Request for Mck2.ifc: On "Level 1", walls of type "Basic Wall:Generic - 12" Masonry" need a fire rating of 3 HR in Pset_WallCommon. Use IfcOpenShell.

First a look at what the model holds.

```python
import ifcopenshell
import ifcopenshell.util.element

model = ifcopenshell.open("Mck2.ifc")
print(model.schema)
storey = next(s for s in model.by_type("IfcBuildingStorey") if s.Name == "Level 1")
walls = [e for e in ifcopenshell.util.element.get_decomposition(storey) if e.is_a("IfcWall")]
seen = {}
for e in walls:
    element_type = ifcopenshell.util.element.get_type(e)
    key = (element_type.Name if element_type != e and element_type else None, ifcopenshell.util.element.get_pset(e, "Pset_WallCommon", "FireRating"))
    seen[key] = seen.get(key, 0) + 1
for (name, value), count in sorted(seen.items(), key=str):
    print(count, "x", name, "|", value)
```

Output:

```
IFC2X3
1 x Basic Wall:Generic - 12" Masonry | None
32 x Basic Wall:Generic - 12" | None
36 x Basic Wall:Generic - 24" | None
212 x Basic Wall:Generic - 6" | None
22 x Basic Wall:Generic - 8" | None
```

```python
import ifcopenshell
import ifcopenshell.api.pset
import ifcopenshell.util.element

model = ifcopenshell.open("Mck2.ifc")

storey = next(s for s in model.by_type("IfcBuildingStorey") if s.Name == "Level 1")
walls = [e for e in ifcopenshell.util.element.get_decomposition(storey) if e.is_a("IfcWall")]

count = 0
for e in walls:
    element_type = ifcopenshell.util.element.get_type(e)
    if element_type in (None, e) or element_type.Name != 'Basic Wall:Generic - 12" Masonry':
        continue
    # add_pset returns the element's existing set when there is one.
    pset = ifcopenshell.api.pset.add_pset(model, product=e, name="Pset_WallCommon")
    ifcopenshell.api.pset.edit_pset(model, pset=pset, properties={"FireRating": "3 HR"})
    count += 1

print(count, "walls updated")

model.write("Mck2-out.ifc")
```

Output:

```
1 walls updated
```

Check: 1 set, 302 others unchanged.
